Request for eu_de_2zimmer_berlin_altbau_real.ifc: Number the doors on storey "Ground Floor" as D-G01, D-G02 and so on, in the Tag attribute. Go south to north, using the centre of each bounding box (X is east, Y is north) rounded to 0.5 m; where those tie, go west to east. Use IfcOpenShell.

First a look at what the model holds.

```python
import ifcopenshell
import ifcopenshell.util.element
import ifcopenshell.util.placement

model = ifcopenshell.open("eu_de_2zimmer_berlin_altbau_real.ifc")
print(model.schema)
storey = next(s for s in model.by_type("IfcBuildingStorey") if s.Name == "Ground Floor")
doors = [e for e in ifcopenshell.util.element.get_decomposition(storey) if e.is_a("IfcDoor")]
for e in sorted(doors, key=lambda e: e.id()):
    origin = ifcopenshell.util.placement.get_local_placement(e.ObjectPlacement)[:3, 3]
    print(e.id(), e.Tag, e.Name, origin.round(2) + 0.0, sep=" | ")
```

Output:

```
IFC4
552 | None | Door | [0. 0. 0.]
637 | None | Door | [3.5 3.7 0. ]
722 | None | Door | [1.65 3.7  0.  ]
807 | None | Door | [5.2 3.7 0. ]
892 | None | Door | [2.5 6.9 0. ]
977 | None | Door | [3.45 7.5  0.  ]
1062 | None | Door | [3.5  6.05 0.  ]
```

```python
import ifcopenshell
import ifcopenshell.geom
import ifcopenshell.util.element
import ifcopenshell.util.shape

model = ifcopenshell.open("eu_de_2zimmer_berlin_altbau_real.ifc")
settings = ifcopenshell.geom.settings()
settings.set("use-world-coords", True)


def centre(element):
    shape = ifcopenshell.geom.create_shape(settings, element)
    return ifcopenshell.util.shape.get_bbox_centroid(shape.geometry)


storey = next(s for s in model.by_type("IfcBuildingStorey") if s.Name == "Ground Floor")
doors = [e for e in ifcopenshell.util.element.get_decomposition(storey) if e.is_a("IfcDoor")]

# Insertion points can sit at a corner or the storey origin, so sort by the geometry (in metres).
centres = {e: centre(e) for e in doors}
doors.sort(key=lambda e: (round(centres[e][1] / 0.5), centres[e][0]))

for i, e in enumerate(doors, start=1):
    number = f"D-G{i:02d}"
    e.Tag = number
    print(e.id(), number)

model.write("eu_de_2zimmer_berlin_altbau_real-out.ifc")
```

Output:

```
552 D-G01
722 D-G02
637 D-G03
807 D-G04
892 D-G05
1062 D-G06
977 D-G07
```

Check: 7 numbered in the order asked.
